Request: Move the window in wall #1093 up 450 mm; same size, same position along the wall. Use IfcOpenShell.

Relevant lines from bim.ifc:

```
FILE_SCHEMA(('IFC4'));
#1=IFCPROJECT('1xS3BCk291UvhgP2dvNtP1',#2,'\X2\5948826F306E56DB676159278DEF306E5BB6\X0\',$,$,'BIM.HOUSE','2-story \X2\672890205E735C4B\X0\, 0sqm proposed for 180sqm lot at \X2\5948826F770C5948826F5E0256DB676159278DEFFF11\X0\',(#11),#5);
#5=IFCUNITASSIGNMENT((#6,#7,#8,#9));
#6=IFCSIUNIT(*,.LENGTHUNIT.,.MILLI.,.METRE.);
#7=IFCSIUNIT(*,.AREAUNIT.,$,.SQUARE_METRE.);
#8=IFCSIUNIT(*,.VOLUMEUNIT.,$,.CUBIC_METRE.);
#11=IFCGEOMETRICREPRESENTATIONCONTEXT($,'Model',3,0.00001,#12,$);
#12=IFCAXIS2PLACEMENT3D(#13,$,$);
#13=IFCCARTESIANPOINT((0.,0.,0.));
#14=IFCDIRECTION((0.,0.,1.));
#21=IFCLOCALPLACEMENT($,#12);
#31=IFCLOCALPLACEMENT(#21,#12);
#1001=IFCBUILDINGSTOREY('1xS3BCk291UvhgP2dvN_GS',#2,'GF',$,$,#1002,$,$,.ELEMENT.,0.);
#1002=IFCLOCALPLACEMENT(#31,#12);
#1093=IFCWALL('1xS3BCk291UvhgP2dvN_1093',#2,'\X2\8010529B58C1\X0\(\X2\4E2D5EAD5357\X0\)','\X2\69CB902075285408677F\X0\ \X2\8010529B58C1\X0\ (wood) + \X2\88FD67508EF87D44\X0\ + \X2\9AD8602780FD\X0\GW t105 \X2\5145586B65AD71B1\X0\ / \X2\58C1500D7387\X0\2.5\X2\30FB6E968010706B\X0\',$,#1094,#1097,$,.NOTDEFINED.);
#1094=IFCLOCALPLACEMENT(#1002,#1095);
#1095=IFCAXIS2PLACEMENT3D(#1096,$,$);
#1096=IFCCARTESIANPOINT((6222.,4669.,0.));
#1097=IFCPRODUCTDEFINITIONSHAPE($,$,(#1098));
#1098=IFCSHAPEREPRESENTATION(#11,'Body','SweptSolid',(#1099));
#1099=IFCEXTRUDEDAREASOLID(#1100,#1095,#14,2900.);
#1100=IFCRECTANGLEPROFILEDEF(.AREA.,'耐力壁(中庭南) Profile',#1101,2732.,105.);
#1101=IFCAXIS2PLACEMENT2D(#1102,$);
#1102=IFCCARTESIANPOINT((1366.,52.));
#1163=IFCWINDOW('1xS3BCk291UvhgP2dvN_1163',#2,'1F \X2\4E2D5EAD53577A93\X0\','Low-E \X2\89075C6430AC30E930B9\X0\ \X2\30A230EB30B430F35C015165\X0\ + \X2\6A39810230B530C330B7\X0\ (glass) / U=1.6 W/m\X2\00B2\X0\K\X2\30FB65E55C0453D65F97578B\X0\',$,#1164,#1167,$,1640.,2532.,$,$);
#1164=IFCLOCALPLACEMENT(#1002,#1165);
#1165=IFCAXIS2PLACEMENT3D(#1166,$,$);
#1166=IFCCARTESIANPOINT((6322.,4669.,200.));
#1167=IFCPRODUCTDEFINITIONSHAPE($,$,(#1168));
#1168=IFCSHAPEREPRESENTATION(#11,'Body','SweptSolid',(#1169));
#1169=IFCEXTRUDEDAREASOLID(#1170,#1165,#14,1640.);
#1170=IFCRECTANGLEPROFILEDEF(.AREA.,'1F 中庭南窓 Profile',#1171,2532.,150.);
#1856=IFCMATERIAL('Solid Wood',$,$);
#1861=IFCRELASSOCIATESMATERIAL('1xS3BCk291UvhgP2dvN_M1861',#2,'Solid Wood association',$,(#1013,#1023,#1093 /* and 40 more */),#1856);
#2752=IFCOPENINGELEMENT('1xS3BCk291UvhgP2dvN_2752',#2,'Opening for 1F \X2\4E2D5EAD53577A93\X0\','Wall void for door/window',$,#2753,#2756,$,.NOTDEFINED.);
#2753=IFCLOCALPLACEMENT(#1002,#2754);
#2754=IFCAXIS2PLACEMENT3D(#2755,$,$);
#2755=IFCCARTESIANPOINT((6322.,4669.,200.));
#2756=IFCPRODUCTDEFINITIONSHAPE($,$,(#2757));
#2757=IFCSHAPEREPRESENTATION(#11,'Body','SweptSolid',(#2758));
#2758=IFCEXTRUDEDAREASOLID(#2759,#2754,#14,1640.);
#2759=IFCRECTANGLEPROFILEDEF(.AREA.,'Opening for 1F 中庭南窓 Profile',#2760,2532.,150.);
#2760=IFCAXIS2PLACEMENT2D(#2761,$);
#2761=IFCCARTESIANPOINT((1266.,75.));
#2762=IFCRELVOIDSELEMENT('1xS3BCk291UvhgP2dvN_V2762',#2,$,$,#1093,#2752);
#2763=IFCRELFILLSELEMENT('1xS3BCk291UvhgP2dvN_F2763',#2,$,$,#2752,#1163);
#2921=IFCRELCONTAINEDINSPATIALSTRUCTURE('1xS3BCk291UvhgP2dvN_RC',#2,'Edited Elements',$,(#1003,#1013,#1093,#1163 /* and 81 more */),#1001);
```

```python
import numpy as np
import ifcopenshell
import ifcopenshell.api.geometry
import ifcopenshell.util.placement
import ifcopenshell.util.unit

model = ifcopenshell.open("bim.ifc")
unit_scale = ifcopenshell.util.unit.calculate_unit_scale(model)

window = model.by_guid("1xS3BCk291UvhgP2dvN_1163")
opening = window.FillsVoids[0].RelatingOpeningElement
dz = 0.45 / unit_scale

shift = np.array([0.0, 0.0, dz])
# The window is not placed relative to its opening, so move both.
for product in (opening, window):
    matrix = ifcopenshell.util.placement.get_local_placement(product.ObjectPlacement)
    matrix[:3, 3] += shift
    ifcopenshell.api.geometry.edit_object_placement(model, product=product, matrix=matrix, is_si=False)

print(f"moved by {dz * unit_scale:+.3f} m")

model.write("bim_updated.ifc")
```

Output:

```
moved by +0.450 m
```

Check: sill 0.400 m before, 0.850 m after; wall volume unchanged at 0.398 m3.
